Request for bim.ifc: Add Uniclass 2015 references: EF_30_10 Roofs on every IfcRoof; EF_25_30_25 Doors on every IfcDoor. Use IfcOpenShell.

First a look at what the model holds.

```python
import ifcopenshell

model = ifcopenshell.open("bim.ifc")
print(model.schema)
print("classifications:", [c.Name for c in model.by_type("IfcClassification")])
for ifc_class in ("IfcDoor", "IfcRoof", "IfcStair", "IfcWall", "IfcWindow"):
    print(ifc_class, len(model.by_type(ifc_class)))
```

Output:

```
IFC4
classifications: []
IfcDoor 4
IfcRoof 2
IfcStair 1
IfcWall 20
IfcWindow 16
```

```python
import ifcopenshell
import ifcopenshell.api.classification

model = ifcopenshell.open("bim.ifc")

system = ifcopenshell.api.classification.add_classification(model, classification="Uniclass 2015")

codes = {
    "IfcRoof": ("EF_30_10", "Roofs"),
    "IfcDoor": ("EF_25_30_25", "Doors"),
}
for ifc_class, (code, name) in codes.items():
    products = model.by_type(ifc_class)
    ifcopenshell.api.classification.add_reference(
        model, products=products, classification=system, identification=code, name=name
    )
    print(code, len(products))

model.write("bim_updated.ifc")
```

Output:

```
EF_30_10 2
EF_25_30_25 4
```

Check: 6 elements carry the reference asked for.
